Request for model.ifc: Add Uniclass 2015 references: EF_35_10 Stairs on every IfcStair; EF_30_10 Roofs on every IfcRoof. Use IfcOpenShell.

First a look at what the model holds.

```python
import ifcopenshell

model = ifcopenshell.open("model.ifc")
print(model.schema)
print("classifications:", [c.Name for c in model.by_type("IfcClassification")])
for ifc_class in ("IfcDoor", "IfcRoof", "IfcStair", "IfcWall", "IfcWindow"):
    print(ifc_class, len(model.by_type(ifc_class)))
```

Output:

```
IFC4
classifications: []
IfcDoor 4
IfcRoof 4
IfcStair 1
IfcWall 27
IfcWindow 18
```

```python
import ifcopenshell
import ifcopenshell.api.classification

model = ifcopenshell.open("model.ifc")

system = ifcopenshell.api.classification.add_classification(model, classification="Uniclass 2015")

codes = {
    "IfcStair": ("EF_35_10", "Stairs"),
    "IfcRoof": ("EF_30_10", "Roofs"),
}
for ifc_class, (code, name) in codes.items():
    products = model.by_type(ifc_class)
    ifcopenshell.api.classification.add_reference(
        model, products=products, classification=system, identification=code, name=name
    )
    print(code, len(products))

model.write("model_rev.ifc")
```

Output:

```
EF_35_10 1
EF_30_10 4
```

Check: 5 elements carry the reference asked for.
